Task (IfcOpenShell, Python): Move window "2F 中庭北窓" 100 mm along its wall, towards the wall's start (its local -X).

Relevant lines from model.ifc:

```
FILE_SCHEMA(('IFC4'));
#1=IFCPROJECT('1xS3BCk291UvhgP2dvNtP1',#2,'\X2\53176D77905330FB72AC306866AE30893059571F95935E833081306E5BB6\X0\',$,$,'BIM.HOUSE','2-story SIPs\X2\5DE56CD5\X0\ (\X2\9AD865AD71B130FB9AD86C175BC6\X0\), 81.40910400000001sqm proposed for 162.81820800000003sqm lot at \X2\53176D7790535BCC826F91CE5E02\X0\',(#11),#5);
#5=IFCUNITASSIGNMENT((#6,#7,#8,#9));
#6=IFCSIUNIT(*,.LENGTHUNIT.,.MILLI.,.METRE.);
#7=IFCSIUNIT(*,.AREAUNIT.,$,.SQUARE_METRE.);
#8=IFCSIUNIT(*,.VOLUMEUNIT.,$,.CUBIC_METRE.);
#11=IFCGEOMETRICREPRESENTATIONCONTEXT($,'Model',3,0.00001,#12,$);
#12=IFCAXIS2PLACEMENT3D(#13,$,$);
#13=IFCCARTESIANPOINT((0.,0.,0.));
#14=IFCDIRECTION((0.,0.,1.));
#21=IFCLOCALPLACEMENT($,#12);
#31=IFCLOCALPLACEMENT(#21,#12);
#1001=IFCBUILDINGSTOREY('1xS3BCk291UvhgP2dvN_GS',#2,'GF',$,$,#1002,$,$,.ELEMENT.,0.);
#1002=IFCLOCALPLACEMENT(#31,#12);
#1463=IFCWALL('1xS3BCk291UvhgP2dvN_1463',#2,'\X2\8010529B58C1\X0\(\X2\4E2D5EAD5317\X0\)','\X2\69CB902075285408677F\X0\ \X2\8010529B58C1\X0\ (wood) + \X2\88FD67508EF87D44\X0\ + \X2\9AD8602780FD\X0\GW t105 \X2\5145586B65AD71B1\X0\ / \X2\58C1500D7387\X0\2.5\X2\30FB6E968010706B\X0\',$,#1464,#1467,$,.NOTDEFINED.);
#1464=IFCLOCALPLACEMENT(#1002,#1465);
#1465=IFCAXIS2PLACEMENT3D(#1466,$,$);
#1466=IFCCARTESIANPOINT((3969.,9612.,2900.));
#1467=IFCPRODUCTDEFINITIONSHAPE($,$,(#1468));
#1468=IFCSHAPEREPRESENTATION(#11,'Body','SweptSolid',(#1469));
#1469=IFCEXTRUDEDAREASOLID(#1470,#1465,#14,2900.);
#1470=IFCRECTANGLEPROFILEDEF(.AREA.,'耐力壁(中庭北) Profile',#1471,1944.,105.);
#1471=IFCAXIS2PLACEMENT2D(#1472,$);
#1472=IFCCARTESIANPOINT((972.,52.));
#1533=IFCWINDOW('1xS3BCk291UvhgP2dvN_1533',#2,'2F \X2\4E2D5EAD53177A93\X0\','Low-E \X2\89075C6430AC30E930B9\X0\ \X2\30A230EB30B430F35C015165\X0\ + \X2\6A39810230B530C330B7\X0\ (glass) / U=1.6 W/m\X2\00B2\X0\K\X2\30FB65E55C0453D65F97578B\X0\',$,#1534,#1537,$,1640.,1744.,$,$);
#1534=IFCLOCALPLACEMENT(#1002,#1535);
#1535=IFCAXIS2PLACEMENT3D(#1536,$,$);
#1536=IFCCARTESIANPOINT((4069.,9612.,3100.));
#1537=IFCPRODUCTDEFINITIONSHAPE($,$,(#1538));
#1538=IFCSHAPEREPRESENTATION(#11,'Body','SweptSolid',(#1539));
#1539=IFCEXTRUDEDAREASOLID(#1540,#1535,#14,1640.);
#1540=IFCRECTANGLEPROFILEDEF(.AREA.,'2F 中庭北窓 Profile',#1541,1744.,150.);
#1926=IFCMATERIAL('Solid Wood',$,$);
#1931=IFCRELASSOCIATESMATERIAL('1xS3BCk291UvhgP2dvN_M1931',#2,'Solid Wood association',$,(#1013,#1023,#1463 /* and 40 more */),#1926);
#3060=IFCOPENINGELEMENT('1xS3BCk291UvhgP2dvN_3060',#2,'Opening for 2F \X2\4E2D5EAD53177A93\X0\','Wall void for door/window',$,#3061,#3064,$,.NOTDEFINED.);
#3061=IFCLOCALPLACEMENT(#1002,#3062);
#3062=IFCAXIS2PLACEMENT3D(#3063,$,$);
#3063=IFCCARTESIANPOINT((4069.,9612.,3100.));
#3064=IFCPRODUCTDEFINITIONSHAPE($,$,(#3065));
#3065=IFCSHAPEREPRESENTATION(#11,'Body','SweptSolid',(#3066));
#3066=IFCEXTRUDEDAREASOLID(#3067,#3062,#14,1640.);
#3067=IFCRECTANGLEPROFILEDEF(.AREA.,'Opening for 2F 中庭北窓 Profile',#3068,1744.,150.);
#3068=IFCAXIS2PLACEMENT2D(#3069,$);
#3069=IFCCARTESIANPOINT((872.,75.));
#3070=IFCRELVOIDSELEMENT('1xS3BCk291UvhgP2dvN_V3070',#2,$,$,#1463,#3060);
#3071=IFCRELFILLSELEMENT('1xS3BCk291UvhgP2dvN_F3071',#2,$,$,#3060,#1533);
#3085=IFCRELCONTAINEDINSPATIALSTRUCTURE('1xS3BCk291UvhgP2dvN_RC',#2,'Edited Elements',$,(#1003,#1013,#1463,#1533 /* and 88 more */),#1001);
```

```python
import ifcopenshell
import ifcopenshell.api.geometry
import ifcopenshell.util.placement

model = ifcopenshell.open("model.ifc")

window = model.by_guid("1xS3BCk291UvhgP2dvN_1533")
opening = window.FillsVoids[0].RelatingOpeningElement
wall = opening.VoidsElements[0].RelatingBuildingElement

wall_matrix = ifcopenshell.util.placement.get_local_placement(wall.ObjectPlacement)
shift = wall_matrix[:3, 0] * -100.0
before = ifcopenshell.util.placement.get_local_placement(window.ObjectPlacement)[:3, 3].copy()

# The window is not placed relative to its opening, so move both.
for product in (opening, window):
    matrix = ifcopenshell.util.placement.get_local_placement(product.ObjectPlacement)
    matrix[:3, 3] += shift
    ifcopenshell.api.geometry.edit_object_placement(model, product=product, matrix=matrix, is_si=False)

after = ifcopenshell.util.placement.get_local_placement(window.ObjectPlacement)[:3, 3]
print("window moved by", (after - before).round(3) + 0.0)

model.write("model_v2.ifc")
```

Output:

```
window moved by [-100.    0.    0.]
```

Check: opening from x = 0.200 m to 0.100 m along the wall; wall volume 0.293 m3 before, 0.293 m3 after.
